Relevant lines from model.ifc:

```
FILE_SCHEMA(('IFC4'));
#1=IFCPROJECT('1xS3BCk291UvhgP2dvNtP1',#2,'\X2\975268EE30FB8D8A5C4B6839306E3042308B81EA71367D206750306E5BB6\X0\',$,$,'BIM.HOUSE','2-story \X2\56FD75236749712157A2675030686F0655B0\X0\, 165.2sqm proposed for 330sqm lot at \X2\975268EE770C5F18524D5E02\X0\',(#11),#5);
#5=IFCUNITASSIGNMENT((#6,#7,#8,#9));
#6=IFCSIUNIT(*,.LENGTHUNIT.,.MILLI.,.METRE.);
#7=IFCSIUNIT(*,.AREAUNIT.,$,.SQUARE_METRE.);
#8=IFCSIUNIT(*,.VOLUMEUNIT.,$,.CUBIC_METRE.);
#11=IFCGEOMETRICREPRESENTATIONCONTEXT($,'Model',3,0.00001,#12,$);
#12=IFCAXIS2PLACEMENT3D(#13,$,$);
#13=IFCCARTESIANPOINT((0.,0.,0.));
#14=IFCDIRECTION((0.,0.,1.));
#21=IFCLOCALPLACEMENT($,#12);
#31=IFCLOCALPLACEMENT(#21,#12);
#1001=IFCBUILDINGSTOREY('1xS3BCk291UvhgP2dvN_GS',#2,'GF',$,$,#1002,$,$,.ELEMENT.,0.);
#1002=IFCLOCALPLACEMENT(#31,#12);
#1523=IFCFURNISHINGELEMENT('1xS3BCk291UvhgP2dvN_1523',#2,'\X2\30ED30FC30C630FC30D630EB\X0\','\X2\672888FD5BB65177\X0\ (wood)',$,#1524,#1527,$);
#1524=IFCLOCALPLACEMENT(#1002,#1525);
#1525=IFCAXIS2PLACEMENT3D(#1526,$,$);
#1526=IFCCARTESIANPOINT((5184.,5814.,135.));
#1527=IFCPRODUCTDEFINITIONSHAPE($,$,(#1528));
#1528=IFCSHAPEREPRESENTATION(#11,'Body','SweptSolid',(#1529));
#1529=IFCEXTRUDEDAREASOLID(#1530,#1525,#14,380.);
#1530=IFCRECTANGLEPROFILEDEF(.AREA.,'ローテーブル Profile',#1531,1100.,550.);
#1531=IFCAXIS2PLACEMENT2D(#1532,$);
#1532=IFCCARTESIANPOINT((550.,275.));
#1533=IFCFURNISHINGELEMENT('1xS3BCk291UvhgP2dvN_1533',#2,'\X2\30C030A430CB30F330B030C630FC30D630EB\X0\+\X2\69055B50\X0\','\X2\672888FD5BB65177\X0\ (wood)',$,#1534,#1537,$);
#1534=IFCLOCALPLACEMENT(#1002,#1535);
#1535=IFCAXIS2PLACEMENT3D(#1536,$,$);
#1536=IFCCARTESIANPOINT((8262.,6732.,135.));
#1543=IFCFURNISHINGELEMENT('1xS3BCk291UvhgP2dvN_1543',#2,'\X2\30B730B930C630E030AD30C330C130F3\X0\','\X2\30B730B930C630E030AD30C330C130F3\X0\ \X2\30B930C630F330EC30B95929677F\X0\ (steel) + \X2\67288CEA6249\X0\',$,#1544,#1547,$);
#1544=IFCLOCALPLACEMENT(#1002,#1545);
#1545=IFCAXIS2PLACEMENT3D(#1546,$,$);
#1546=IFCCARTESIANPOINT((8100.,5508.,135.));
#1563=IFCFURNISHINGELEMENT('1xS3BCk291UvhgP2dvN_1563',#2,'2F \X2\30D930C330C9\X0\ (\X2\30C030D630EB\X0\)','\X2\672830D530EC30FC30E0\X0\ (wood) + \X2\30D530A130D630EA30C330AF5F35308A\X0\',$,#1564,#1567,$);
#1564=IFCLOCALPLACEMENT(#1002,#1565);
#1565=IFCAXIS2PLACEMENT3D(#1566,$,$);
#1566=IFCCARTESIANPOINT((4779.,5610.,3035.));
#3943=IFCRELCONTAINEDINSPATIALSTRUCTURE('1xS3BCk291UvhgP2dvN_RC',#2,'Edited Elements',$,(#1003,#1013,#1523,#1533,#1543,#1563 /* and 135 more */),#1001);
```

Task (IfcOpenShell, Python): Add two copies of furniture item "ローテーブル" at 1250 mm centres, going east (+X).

```python
import numpy as np
import ifcopenshell
import ifcopenshell.api.geometry
import ifcopenshell.api.root
import ifcopenshell.util.element
import ifcopenshell.util.placement

model = ifcopenshell.open("model.ifc")


def reuse_history(source, copy):
    """copy_class also copies each property set's owner history, people and application; keep the originals."""
    for rel in copy.IsDefinedBy:
        if rel.is_a("IfcRelDefinesByProperties") and (history := rel.RelatingPropertyDefinition.OwnerHistory):
            rel.RelatingPropertyDefinition.OwnerHistory = source.OwnerHistory
            ifcopenshell.util.element.remove_deep2(model, history)


source = model.by_id(1523)
base = ifcopenshell.util.placement.get_local_placement(source.ObjectPlacement)
step = np.array([1.0, 0.0, 0.0]) * 1250.0

for i in range(1, 3):
    copy = ifcopenshell.api.root.copy_class(model, product=source)
    copy.Representation = ifcopenshell.util.element.copy_deep(
        model, source.Representation, exclude=["IfcGeometricRepresentationContext", "IfcRepresentationMap"]
    )
    reuse_history(source, copy)
    matrix = base.copy()
    matrix[:3, 3] += i * step
    print("added at", matrix[:3, 3].round(3) + 0.0)
    ifcopenshell.api.geometry.edit_object_placement(model, product=copy, matrix=matrix, is_si=False)

model.write("model_rev.ifc")
```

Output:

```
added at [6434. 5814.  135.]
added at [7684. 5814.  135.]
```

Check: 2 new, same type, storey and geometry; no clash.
